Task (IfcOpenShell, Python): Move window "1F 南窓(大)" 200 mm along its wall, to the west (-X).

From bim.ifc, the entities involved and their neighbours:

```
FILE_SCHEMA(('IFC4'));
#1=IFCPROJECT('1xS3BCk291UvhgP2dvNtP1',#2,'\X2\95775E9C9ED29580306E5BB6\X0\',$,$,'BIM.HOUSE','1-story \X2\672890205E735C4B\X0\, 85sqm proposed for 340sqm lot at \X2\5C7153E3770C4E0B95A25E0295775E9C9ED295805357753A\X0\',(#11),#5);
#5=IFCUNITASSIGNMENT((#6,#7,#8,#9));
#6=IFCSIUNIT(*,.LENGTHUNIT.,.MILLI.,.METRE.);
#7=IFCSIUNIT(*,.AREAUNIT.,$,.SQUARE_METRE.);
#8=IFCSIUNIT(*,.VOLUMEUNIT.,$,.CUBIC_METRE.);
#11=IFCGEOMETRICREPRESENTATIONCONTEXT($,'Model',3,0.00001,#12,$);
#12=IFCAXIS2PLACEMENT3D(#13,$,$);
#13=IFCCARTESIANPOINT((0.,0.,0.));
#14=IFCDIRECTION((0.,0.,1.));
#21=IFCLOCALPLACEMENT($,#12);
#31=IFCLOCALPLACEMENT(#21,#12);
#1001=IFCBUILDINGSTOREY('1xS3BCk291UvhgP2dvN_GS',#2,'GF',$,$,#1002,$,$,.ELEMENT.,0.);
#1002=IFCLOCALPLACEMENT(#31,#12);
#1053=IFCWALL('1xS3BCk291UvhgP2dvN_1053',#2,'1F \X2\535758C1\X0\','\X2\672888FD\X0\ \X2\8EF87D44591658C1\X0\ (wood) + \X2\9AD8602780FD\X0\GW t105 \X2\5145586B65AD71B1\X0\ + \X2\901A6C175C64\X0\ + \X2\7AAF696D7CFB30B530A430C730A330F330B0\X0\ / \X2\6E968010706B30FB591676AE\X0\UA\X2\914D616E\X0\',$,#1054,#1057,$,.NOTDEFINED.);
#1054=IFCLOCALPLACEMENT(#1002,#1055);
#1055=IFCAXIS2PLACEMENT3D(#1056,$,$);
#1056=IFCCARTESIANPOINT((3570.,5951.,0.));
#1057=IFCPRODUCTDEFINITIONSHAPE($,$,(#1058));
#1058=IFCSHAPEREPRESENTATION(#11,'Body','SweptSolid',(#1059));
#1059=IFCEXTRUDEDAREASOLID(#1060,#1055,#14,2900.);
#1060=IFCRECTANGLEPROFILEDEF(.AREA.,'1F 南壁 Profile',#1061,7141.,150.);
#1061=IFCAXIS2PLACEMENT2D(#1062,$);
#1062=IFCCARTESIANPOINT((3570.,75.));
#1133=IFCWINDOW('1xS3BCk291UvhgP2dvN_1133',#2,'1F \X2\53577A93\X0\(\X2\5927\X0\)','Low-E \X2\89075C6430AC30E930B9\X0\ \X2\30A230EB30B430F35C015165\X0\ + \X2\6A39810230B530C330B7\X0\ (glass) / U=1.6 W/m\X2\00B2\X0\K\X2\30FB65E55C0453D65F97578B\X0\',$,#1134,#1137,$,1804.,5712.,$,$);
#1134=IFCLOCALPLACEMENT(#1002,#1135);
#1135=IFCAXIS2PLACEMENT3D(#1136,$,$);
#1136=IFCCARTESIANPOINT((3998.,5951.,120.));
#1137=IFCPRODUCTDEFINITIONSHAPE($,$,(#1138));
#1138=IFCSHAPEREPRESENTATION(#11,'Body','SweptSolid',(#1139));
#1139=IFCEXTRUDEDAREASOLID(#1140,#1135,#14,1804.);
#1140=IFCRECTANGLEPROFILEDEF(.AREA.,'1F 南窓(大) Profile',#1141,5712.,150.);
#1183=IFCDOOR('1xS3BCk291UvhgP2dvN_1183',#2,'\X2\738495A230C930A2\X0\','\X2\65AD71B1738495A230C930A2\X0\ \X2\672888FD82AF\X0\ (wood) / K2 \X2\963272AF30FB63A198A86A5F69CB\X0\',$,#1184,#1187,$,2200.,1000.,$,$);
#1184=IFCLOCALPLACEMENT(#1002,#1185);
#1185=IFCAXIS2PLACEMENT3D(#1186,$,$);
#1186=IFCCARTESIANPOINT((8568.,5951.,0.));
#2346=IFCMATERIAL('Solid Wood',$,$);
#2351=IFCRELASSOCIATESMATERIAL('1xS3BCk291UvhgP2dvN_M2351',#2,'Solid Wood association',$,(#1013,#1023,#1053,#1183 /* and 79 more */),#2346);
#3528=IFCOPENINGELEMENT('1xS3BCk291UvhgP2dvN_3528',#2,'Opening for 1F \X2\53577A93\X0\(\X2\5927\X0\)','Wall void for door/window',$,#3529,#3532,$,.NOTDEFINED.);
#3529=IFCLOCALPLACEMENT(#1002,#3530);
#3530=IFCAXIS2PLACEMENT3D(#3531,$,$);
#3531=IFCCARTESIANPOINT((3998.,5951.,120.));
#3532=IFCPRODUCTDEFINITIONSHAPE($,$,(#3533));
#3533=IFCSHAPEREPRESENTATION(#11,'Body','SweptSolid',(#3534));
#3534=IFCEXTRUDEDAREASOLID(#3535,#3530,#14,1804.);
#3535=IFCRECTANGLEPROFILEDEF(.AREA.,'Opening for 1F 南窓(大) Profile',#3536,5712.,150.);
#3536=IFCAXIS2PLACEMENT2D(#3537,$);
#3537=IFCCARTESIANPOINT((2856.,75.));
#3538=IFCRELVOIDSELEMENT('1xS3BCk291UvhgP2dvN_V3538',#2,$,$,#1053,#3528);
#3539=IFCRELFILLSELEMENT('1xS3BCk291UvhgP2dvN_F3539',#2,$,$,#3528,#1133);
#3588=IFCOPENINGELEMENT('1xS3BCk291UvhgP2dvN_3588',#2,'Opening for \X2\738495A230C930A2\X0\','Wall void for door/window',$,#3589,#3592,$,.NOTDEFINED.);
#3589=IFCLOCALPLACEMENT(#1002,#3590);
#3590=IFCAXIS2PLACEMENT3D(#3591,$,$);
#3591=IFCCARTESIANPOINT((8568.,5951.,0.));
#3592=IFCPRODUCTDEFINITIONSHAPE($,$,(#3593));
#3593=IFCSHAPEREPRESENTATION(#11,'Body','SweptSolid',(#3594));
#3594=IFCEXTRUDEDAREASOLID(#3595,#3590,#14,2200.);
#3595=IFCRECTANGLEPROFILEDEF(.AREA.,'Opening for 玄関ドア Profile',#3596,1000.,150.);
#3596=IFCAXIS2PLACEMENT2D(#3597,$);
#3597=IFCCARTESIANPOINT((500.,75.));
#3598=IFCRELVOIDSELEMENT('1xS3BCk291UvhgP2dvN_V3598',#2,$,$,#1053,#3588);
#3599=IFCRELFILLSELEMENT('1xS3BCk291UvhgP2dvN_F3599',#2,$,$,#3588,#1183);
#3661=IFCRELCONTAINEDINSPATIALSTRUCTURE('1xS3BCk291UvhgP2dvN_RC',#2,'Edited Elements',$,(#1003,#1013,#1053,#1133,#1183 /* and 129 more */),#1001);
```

```python
import ifcopenshell
import ifcopenshell.api.geometry
import ifcopenshell.util.placement
import ifcopenshell.util.unit

model = ifcopenshell.open("bim.ifc")
unit_scale = ifcopenshell.util.unit.calculate_unit_scale(model)

window = model.by_guid("1xS3BCk291UvhgP2dvN_1133")
opening = window.FillsVoids[0].RelatingOpeningElement
wall = opening.VoidsElements[0].RelatingBuildingElement

wall_matrix = ifcopenshell.util.placement.get_local_placement(wall.ObjectPlacement)
shift = wall_matrix[:3, 0] * -0.2 / unit_scale
before = ifcopenshell.util.placement.get_local_placement(window.ObjectPlacement)[:3, 3].copy()

# The window is not placed relative to its opening, so move both.
for product in (opening, window):
    matrix = ifcopenshell.util.placement.get_local_placement(product.ObjectPlacement)
    matrix[:3, 3] += shift
    ifcopenshell.api.geometry.edit_object_placement(model, product=product, matrix=matrix, is_si=False)

after = ifcopenshell.util.placement.get_local_placement(window.ObjectPlacement)[:3, 3]
print("window moved by", (after - before).round(3) + 0.0)

model.write("bim_edited.ifc")
```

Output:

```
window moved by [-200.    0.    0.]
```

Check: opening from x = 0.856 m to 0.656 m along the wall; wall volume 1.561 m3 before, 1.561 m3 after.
